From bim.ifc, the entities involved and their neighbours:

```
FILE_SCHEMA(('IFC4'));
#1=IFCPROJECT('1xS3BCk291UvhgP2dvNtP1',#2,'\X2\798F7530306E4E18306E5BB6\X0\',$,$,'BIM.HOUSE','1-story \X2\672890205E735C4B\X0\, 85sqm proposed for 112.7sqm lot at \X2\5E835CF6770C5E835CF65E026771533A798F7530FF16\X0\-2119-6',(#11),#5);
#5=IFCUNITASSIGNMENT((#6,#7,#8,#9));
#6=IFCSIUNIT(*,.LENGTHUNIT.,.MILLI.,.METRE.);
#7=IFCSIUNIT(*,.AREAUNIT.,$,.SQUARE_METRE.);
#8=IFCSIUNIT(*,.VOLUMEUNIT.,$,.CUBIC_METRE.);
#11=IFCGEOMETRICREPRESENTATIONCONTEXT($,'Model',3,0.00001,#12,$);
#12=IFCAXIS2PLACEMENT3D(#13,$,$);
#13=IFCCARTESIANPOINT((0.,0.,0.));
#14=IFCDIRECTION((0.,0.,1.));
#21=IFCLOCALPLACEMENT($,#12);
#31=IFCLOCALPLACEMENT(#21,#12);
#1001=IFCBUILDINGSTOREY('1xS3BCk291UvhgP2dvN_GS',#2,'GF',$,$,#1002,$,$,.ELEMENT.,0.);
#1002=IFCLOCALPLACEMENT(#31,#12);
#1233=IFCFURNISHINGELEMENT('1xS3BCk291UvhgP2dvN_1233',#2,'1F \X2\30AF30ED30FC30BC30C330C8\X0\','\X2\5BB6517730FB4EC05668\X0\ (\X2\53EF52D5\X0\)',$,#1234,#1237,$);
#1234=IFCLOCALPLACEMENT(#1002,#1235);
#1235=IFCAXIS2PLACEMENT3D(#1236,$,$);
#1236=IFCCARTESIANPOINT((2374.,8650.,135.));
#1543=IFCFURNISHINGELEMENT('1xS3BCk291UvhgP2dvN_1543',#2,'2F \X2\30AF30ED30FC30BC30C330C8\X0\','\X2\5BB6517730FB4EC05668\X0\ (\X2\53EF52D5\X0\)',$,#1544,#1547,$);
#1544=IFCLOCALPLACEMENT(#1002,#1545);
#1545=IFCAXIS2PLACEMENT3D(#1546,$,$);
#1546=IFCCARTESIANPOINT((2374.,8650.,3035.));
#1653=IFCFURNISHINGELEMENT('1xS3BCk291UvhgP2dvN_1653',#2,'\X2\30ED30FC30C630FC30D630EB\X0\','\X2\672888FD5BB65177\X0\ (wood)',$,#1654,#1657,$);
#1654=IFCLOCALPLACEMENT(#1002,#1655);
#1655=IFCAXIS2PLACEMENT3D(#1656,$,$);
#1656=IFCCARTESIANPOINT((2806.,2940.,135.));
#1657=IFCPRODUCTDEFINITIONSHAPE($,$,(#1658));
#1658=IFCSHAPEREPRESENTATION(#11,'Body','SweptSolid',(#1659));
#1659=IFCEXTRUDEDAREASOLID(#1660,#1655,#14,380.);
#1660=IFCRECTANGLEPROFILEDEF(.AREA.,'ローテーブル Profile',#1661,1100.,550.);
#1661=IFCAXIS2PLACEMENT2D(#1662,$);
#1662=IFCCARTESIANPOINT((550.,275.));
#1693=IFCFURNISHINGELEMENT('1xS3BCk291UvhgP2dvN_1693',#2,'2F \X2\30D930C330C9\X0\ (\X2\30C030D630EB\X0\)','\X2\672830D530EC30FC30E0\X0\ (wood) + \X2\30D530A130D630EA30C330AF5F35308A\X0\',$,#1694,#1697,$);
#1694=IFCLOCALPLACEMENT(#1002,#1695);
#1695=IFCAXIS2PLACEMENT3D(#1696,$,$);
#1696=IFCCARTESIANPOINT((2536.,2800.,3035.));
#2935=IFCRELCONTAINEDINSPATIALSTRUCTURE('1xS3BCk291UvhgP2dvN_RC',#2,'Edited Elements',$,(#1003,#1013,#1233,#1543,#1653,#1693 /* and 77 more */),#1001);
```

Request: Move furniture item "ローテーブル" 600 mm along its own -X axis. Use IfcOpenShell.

```python
import ifcopenshell
import ifcopenshell.api.geometry
import ifcopenshell.util.placement
import ifcopenshell.util.unit

model = ifcopenshell.open("bim.ifc")
unit_scale = ifcopenshell.util.unit.calculate_unit_scale(model)

item = model.by_id(1653)
matrix = ifcopenshell.util.placement.get_local_placement(item.ObjectPlacement)
matrix[:3, 3] -= matrix[:3, 0] * 0.6 / unit_scale
ifcopenshell.api.geometry.edit_object_placement(model, product=item, matrix=matrix, is_si=False)

print(ifcopenshell.util.placement.get_local_placement(item.ObjectPlacement).round(3) + 0.0)

model.write("bim_edited.ifc")
```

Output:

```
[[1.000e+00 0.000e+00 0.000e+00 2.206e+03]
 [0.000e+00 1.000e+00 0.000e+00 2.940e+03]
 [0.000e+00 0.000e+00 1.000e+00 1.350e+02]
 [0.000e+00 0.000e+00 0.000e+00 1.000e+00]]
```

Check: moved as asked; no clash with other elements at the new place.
